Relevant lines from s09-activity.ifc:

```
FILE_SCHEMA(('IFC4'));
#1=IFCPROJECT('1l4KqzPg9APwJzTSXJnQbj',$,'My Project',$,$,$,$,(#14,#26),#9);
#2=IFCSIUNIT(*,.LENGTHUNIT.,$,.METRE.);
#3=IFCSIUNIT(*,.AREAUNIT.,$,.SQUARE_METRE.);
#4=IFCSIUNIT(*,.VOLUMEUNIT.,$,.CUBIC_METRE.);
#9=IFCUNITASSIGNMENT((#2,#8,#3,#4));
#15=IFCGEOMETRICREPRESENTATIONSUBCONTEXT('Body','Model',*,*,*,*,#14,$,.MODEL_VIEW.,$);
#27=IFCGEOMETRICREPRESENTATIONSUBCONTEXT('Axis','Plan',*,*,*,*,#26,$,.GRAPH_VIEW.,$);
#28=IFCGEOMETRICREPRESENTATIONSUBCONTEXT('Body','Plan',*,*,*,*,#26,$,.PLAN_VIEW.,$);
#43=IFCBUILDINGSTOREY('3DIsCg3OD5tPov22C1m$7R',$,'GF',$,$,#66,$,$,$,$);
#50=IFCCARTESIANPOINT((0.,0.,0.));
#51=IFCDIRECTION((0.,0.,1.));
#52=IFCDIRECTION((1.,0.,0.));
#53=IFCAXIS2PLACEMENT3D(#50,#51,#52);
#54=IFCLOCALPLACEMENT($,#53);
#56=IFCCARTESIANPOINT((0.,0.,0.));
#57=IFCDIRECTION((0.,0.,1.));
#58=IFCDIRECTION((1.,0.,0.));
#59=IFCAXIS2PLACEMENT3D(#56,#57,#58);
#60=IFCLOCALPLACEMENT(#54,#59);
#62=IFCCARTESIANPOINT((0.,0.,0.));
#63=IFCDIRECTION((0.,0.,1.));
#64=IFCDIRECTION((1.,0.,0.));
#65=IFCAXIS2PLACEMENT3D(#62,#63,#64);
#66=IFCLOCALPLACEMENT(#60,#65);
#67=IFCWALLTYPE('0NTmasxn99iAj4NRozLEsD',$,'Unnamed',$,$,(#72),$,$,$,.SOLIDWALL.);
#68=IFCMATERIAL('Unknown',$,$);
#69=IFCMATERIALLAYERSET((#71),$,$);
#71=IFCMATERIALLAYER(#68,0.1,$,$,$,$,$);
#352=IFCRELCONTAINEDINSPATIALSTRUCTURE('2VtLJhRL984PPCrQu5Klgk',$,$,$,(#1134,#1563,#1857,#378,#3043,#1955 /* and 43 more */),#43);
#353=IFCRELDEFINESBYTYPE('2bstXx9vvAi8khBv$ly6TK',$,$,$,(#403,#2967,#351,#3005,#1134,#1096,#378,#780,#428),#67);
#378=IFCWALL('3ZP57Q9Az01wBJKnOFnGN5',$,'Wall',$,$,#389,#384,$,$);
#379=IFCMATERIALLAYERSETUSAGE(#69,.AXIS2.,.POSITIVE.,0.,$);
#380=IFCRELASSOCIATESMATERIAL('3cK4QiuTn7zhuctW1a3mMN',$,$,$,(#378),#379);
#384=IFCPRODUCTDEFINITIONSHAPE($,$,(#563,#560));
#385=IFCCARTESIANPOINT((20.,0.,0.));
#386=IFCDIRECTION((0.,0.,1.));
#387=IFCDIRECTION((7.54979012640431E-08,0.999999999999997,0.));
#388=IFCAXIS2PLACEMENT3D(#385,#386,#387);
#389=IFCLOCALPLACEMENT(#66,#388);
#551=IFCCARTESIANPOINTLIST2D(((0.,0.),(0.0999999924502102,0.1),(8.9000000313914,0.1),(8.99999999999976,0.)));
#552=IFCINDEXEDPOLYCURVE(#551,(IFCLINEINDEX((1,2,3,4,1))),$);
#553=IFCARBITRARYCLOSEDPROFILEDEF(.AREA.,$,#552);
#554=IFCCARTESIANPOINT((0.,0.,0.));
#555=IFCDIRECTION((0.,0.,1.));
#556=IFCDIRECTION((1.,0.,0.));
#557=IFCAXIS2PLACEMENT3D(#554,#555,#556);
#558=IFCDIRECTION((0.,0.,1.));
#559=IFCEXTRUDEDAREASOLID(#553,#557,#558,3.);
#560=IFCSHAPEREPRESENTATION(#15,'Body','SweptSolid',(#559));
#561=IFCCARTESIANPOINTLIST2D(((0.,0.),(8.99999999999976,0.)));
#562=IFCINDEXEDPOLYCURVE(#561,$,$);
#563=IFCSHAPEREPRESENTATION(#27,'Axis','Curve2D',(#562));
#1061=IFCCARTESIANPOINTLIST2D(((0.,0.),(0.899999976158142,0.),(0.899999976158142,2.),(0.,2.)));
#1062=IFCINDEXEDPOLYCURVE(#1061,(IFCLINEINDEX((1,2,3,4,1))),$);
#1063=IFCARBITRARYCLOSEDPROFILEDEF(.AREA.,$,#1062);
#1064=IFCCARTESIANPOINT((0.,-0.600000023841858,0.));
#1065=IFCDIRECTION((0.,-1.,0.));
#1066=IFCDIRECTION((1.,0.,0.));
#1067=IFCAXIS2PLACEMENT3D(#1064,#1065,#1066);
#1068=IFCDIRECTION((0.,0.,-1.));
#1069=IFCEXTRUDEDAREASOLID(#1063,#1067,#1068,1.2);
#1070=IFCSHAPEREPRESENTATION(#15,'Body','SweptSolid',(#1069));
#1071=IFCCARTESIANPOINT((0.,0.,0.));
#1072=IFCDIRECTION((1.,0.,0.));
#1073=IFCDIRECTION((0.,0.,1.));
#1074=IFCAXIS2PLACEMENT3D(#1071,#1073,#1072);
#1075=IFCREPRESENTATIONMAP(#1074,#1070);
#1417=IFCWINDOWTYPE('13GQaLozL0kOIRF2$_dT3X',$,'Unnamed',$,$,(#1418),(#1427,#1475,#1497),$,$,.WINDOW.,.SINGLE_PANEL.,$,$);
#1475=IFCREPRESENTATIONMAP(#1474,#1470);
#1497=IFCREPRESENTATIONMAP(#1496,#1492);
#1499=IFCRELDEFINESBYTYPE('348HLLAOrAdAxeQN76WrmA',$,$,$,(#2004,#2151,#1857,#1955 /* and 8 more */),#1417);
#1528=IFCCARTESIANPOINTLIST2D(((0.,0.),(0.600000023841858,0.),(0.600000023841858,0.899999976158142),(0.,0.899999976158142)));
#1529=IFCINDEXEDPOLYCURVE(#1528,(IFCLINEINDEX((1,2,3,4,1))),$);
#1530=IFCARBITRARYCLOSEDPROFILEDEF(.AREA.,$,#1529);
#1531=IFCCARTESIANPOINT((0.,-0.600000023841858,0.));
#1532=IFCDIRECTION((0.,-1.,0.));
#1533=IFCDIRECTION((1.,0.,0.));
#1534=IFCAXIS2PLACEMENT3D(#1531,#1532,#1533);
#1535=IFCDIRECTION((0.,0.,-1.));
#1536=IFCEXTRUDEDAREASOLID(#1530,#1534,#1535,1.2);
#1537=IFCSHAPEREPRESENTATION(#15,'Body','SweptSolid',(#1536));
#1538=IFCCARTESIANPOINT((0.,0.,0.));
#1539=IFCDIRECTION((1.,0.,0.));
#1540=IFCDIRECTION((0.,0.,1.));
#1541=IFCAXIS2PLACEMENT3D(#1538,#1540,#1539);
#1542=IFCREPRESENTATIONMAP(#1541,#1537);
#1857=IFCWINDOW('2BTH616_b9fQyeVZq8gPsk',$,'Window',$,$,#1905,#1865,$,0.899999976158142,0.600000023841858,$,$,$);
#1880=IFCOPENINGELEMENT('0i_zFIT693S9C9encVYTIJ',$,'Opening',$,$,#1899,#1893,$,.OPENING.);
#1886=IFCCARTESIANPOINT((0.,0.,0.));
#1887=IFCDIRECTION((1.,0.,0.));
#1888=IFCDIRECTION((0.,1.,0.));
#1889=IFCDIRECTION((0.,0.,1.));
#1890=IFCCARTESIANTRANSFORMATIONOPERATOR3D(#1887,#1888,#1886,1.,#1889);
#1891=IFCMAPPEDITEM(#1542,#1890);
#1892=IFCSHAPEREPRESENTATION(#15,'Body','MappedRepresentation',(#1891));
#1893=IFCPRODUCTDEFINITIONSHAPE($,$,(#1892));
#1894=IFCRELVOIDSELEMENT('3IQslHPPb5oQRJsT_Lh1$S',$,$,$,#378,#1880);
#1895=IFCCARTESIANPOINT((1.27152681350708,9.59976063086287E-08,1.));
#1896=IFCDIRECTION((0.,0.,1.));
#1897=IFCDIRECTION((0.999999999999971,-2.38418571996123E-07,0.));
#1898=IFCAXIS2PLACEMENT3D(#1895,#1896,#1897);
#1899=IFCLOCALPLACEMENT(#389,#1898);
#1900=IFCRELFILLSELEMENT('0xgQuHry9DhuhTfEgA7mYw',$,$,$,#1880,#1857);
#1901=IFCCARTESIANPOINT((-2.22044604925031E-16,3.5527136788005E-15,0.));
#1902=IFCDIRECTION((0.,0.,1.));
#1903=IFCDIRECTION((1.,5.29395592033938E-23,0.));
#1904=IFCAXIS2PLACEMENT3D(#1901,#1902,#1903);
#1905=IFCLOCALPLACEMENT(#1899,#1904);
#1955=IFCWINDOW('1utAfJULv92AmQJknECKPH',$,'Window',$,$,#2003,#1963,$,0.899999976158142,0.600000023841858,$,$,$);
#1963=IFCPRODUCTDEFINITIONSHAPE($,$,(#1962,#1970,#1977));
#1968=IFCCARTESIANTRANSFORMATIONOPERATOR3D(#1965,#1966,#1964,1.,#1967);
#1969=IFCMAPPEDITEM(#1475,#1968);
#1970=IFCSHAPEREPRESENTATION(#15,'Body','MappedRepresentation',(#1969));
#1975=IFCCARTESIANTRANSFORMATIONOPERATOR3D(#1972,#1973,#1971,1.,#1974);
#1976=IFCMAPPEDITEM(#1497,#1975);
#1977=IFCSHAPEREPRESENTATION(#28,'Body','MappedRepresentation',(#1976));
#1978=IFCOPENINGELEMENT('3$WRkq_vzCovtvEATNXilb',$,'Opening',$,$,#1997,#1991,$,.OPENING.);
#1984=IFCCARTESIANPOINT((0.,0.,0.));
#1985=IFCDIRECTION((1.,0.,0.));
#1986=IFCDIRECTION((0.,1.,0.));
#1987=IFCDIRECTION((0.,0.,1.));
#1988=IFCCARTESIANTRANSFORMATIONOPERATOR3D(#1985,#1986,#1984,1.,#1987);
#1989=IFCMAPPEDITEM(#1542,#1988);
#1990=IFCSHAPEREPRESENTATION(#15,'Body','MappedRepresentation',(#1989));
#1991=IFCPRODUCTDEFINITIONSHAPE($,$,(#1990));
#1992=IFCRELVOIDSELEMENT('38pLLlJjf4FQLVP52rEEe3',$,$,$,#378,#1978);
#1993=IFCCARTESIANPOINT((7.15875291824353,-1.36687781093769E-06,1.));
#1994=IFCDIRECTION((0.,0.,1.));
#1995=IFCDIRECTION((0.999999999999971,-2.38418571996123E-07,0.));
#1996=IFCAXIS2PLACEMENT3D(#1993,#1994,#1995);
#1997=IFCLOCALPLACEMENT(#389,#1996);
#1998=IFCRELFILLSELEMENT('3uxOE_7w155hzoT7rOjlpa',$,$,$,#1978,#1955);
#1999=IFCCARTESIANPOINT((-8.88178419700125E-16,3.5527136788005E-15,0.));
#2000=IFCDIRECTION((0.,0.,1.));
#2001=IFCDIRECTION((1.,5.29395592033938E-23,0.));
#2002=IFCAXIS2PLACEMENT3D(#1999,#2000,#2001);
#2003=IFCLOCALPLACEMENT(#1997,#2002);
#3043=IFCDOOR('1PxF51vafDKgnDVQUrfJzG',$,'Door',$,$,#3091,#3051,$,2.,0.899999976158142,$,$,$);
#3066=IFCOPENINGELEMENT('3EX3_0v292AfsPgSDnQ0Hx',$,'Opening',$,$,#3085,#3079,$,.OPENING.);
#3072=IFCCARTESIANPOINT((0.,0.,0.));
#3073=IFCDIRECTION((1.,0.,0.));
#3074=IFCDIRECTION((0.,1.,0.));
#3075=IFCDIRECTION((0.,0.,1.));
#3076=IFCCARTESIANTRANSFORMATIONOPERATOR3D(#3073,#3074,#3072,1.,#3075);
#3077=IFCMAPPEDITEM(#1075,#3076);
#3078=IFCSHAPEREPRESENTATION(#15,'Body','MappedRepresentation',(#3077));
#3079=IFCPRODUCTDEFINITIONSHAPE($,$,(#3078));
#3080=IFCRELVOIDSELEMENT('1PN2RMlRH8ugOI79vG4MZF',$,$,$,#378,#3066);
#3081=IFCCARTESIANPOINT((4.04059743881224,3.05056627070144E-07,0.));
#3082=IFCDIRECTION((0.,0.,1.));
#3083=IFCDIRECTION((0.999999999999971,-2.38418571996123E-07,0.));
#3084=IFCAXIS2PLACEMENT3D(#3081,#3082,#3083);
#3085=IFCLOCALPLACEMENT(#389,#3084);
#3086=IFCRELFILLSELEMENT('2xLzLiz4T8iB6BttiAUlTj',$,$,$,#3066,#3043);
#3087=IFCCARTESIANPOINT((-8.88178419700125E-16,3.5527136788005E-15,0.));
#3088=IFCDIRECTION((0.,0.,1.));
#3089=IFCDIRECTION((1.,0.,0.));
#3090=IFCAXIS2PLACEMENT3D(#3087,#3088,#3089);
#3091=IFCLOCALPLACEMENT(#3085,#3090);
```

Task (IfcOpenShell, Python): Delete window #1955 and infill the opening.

```python
import ifcopenshell
import ifcopenshell.api.feature
import ifcopenshell.api.root
import ifcopenshell.geom
import ifcopenshell.util.shape

model = ifcopenshell.open("s09-activity.ifc")
settings = ifcopenshell.geom.settings()


def volume(element):
    """Net volume in cubic metres, openings subtracted."""
    shape = ifcopenshell.geom.create_shape(settings, element)
    return ifcopenshell.util.shape.get_volume(shape.geometry)


window = model.by_guid("1utAfJULv92AmQJknECKPH")
opening = window.FillsVoids[0].RelatingOpeningElement
wall = opening.VoidsElements[0].RelatingBuildingElement
before = volume(wall)

ifcopenshell.api.root.remove_product(model, product=window)
ifcopenshell.api.feature.remove_feature(model, feature=opening)

after = volume(wall)

print(f"wall volume {before:.3f} -> {after:.3f} m3")

model.write("s09-activity_updated.ifc")
```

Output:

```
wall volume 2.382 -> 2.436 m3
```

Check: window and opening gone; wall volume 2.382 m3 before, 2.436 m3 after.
